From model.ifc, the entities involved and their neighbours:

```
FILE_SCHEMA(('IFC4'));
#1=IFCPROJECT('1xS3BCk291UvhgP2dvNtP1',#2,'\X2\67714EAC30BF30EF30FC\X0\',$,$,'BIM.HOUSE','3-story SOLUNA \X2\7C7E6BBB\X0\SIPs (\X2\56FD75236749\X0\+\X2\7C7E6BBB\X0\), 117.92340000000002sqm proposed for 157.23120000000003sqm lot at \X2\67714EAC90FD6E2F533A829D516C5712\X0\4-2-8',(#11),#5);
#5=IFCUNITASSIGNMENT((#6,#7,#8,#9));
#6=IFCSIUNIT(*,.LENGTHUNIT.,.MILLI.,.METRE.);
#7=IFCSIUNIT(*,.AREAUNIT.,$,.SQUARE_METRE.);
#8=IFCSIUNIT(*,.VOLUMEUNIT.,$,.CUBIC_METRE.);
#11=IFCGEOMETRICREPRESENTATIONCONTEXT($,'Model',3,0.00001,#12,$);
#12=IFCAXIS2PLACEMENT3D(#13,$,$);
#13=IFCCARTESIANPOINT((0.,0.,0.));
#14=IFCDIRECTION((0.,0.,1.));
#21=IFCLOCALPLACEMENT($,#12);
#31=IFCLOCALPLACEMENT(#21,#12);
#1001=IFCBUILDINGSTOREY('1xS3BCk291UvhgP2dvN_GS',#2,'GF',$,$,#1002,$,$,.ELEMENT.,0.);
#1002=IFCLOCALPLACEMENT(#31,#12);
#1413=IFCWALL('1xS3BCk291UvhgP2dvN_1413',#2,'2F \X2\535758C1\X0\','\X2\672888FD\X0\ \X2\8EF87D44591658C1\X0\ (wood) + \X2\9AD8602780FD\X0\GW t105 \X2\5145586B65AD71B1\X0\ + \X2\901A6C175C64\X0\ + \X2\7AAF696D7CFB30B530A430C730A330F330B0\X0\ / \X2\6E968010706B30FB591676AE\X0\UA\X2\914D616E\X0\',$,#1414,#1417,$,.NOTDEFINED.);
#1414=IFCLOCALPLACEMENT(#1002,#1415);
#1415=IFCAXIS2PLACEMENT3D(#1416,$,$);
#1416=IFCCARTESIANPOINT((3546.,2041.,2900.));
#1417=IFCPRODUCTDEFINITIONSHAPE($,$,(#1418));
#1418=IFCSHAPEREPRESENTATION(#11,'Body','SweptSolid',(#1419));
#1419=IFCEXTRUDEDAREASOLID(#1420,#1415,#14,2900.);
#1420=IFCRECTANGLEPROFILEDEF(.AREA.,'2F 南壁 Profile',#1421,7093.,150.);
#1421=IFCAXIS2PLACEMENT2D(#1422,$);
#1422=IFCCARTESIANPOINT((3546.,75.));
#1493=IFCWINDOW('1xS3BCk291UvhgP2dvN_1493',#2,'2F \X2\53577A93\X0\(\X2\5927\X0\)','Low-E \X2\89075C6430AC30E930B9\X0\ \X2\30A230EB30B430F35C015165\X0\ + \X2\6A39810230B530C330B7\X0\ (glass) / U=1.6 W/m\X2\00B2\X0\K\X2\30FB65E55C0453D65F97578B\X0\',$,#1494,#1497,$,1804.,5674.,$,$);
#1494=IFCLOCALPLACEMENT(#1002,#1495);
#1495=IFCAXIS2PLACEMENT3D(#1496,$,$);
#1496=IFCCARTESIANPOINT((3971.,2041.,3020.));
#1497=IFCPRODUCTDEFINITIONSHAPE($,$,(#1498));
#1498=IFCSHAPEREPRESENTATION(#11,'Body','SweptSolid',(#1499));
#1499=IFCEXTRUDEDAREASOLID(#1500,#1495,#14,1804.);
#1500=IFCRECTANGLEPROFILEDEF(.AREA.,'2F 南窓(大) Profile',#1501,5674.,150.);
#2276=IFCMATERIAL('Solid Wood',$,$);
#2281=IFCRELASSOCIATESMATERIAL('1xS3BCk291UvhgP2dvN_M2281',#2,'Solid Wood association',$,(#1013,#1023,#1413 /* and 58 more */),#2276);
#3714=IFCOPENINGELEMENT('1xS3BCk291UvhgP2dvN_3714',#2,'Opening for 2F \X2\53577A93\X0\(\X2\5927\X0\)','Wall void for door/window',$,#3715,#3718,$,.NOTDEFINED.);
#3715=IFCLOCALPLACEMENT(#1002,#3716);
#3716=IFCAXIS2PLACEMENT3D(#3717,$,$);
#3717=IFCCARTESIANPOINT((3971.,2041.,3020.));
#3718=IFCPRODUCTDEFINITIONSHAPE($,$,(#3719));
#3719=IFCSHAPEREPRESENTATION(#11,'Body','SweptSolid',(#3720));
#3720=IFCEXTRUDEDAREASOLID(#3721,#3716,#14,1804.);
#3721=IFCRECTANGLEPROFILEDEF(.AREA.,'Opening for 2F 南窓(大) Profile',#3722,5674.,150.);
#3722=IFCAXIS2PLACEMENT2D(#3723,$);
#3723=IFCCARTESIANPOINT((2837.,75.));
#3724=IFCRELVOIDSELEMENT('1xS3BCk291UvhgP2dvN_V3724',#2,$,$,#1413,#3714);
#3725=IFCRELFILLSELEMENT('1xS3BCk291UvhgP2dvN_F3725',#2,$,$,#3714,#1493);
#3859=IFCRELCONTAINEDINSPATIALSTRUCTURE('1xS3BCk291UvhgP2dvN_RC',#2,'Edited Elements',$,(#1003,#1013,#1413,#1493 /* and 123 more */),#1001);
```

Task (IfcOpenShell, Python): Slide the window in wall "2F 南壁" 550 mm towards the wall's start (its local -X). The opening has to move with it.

```python
import ifcopenshell
import ifcopenshell.api.geometry
import ifcopenshell.util.placement
import ifcopenshell.util.unit

model = ifcopenshell.open("model.ifc")
unit_scale = ifcopenshell.util.unit.calculate_unit_scale(model)

window = model.by_guid("1xS3BCk291UvhgP2dvN_1493")
opening = window.FillsVoids[0].RelatingOpeningElement
wall = opening.VoidsElements[0].RelatingBuildingElement

wall_matrix = ifcopenshell.util.placement.get_local_placement(wall.ObjectPlacement)
shift = wall_matrix[:3, 0] * -0.55 / unit_scale
before = ifcopenshell.util.placement.get_local_placement(window.ObjectPlacement)[:3, 3].copy()

# The window is not placed relative to its opening, so move both.
for product in (opening, window):
    matrix = ifcopenshell.util.placement.get_local_placement(product.ObjectPlacement)
    matrix[:3, 3] += shift
    ifcopenshell.api.geometry.edit_object_placement(model, product=product, matrix=matrix, is_si=False)

after = ifcopenshell.util.placement.get_local_placement(window.ObjectPlacement)[:3, 3]
print("window moved by", (after - before).round(3) + 0.0)

model.write("model_v2.ifc")
```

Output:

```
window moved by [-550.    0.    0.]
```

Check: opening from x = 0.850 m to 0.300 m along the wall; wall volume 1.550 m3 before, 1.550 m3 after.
